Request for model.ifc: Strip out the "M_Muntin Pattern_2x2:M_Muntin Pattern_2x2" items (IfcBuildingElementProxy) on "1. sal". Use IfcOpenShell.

First a look at what the model holds.

```python
import ifcopenshell
import ifcopenshell.util.element

model = ifcopenshell.open("model.ifc")
print(model.schema)
storey = next(s for s in model.by_type("IfcBuildingStorey") if s.Name == "1. sal")
proxies = [e for e in ifcopenshell.util.element.get_decomposition(storey) if e.is_a("IfcBuildingElementProxy")]
seen = {}
for e in proxies:
    element_type = ifcopenshell.util.element.get_type(e)
    name = element_type.Name if element_type not in (None, e) else None
    seen[name] = seen.get(name, 0) + 1
for name, count in sorted(seen.items(), key=str):
    print(count, "x", name)
```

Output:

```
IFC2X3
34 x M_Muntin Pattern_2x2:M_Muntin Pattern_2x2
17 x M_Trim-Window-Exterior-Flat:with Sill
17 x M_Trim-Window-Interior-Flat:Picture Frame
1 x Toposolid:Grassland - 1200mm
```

```python
import ifcopenshell
import ifcopenshell.api.root
import ifcopenshell.util.element

model = ifcopenshell.open("model.ifc")

storey = next(s for s in model.by_type("IfcBuildingStorey") if s.Name == "1. sal")
proxies = [e for e in ifcopenshell.util.element.get_decomposition(storey) if e.is_a("IfcBuildingElementProxy")]
targets = [e for e in proxies if (t := ifcopenshell.util.element.get_type(e)) not in (None, e) and t.Name == "M_Muntin Pattern_2x2:M_Muntin Pattern_2x2"]

for e in targets:
    ifcopenshell.api.root.remove_product(model, product=e)
print(len(targets), "removed")

model.write("model_rev.ifc")
```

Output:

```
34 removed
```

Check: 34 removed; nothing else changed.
